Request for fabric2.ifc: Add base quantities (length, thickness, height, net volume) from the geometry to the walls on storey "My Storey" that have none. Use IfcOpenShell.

First a look at what the model holds.

```python
import ifcopenshell
import ifcopenshell.util.element
import ifcopenshell.util.unit

model = ifcopenshell.open("fabric2.ifc")
print(model.schema)
for unit_type in ("LENGTHUNIT", "AREAUNIT", "VOLUMEUNIT"):
    print(unit_type, ifcopenshell.util.unit.calculate_unit_scale(model, unit_type))
storey = next(s for s in model.by_type("IfcBuildingStorey") if s.Name == "My Storey")
walls = [e for e in ifcopenshell.util.element.get_decomposition(storey) if e.is_a("IfcWall")]
for e in sorted(walls, key=lambda e: e.id()):
    print(e.id(), e.is_a(), e.Name, list(ifcopenshell.util.element.get_psets(e, qtos_only=True)), sep=" | ")
```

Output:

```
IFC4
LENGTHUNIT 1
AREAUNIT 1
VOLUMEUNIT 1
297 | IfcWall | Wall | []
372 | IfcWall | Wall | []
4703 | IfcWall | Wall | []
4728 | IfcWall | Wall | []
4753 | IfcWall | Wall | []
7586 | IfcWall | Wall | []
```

```python
import ifcopenshell
import ifcopenshell.api.pset
import ifcopenshell.geom
import ifcopenshell.util.element
import ifcopenshell.util.shape
import ifcopenshell.util.unit

model = ifcopenshell.open("fabric2.ifc")
unit_scale = ifcopenshell.util.unit.calculate_unit_scale(model)
volume_scale = ifcopenshell.util.unit.calculate_unit_scale(model, "VOLUMEUNIT")
settings = ifcopenshell.geom.settings()

storey = next(s for s in model.by_type("IfcBuildingStorey") if s.Name == "My Storey")
walls = [e for e in ifcopenshell.util.element.get_decomposition(storey) if e.is_a("IfcWall")]

for e in sorted(walls, key=lambda e: e.id()):
    if ifcopenshell.util.element.get_psets(e, qtos_only=True, should_inherit=False):
        continue
    # Geometry comes back in metres, in the element's own axes.
    shape = ifcopenshell.geom.create_shape(settings, e)
    values = {
        "Length": ifcopenshell.util.shape.get_x(shape.geometry) / unit_scale,
        "Width": ifcopenshell.util.shape.get_y(shape.geometry) / unit_scale,
        "Height": ifcopenshell.util.shape.get_z(shape.geometry) / unit_scale,
        "NetVolume": ifcopenshell.util.shape.get_volume(shape.geometry) / volume_scale,
    }
    qto = ifcopenshell.api.pset.add_qto(model, product=e, name="Qto_WallBaseQuantities")
    ifcopenshell.api.pset.edit_qto(model, qto=qto, properties=values)
    print(e.id(), {k: round(v, 3) for k, v in values.items()})

model.write("fabric2-out.ifc")
```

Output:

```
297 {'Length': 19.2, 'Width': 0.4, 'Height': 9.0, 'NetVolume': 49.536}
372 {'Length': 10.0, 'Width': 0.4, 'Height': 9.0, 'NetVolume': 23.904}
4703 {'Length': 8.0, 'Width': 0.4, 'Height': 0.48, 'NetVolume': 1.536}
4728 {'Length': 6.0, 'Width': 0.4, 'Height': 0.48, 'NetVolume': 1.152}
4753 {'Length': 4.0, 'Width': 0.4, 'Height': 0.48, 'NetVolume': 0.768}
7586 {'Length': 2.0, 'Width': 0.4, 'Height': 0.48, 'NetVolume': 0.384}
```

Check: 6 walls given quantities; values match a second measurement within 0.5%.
